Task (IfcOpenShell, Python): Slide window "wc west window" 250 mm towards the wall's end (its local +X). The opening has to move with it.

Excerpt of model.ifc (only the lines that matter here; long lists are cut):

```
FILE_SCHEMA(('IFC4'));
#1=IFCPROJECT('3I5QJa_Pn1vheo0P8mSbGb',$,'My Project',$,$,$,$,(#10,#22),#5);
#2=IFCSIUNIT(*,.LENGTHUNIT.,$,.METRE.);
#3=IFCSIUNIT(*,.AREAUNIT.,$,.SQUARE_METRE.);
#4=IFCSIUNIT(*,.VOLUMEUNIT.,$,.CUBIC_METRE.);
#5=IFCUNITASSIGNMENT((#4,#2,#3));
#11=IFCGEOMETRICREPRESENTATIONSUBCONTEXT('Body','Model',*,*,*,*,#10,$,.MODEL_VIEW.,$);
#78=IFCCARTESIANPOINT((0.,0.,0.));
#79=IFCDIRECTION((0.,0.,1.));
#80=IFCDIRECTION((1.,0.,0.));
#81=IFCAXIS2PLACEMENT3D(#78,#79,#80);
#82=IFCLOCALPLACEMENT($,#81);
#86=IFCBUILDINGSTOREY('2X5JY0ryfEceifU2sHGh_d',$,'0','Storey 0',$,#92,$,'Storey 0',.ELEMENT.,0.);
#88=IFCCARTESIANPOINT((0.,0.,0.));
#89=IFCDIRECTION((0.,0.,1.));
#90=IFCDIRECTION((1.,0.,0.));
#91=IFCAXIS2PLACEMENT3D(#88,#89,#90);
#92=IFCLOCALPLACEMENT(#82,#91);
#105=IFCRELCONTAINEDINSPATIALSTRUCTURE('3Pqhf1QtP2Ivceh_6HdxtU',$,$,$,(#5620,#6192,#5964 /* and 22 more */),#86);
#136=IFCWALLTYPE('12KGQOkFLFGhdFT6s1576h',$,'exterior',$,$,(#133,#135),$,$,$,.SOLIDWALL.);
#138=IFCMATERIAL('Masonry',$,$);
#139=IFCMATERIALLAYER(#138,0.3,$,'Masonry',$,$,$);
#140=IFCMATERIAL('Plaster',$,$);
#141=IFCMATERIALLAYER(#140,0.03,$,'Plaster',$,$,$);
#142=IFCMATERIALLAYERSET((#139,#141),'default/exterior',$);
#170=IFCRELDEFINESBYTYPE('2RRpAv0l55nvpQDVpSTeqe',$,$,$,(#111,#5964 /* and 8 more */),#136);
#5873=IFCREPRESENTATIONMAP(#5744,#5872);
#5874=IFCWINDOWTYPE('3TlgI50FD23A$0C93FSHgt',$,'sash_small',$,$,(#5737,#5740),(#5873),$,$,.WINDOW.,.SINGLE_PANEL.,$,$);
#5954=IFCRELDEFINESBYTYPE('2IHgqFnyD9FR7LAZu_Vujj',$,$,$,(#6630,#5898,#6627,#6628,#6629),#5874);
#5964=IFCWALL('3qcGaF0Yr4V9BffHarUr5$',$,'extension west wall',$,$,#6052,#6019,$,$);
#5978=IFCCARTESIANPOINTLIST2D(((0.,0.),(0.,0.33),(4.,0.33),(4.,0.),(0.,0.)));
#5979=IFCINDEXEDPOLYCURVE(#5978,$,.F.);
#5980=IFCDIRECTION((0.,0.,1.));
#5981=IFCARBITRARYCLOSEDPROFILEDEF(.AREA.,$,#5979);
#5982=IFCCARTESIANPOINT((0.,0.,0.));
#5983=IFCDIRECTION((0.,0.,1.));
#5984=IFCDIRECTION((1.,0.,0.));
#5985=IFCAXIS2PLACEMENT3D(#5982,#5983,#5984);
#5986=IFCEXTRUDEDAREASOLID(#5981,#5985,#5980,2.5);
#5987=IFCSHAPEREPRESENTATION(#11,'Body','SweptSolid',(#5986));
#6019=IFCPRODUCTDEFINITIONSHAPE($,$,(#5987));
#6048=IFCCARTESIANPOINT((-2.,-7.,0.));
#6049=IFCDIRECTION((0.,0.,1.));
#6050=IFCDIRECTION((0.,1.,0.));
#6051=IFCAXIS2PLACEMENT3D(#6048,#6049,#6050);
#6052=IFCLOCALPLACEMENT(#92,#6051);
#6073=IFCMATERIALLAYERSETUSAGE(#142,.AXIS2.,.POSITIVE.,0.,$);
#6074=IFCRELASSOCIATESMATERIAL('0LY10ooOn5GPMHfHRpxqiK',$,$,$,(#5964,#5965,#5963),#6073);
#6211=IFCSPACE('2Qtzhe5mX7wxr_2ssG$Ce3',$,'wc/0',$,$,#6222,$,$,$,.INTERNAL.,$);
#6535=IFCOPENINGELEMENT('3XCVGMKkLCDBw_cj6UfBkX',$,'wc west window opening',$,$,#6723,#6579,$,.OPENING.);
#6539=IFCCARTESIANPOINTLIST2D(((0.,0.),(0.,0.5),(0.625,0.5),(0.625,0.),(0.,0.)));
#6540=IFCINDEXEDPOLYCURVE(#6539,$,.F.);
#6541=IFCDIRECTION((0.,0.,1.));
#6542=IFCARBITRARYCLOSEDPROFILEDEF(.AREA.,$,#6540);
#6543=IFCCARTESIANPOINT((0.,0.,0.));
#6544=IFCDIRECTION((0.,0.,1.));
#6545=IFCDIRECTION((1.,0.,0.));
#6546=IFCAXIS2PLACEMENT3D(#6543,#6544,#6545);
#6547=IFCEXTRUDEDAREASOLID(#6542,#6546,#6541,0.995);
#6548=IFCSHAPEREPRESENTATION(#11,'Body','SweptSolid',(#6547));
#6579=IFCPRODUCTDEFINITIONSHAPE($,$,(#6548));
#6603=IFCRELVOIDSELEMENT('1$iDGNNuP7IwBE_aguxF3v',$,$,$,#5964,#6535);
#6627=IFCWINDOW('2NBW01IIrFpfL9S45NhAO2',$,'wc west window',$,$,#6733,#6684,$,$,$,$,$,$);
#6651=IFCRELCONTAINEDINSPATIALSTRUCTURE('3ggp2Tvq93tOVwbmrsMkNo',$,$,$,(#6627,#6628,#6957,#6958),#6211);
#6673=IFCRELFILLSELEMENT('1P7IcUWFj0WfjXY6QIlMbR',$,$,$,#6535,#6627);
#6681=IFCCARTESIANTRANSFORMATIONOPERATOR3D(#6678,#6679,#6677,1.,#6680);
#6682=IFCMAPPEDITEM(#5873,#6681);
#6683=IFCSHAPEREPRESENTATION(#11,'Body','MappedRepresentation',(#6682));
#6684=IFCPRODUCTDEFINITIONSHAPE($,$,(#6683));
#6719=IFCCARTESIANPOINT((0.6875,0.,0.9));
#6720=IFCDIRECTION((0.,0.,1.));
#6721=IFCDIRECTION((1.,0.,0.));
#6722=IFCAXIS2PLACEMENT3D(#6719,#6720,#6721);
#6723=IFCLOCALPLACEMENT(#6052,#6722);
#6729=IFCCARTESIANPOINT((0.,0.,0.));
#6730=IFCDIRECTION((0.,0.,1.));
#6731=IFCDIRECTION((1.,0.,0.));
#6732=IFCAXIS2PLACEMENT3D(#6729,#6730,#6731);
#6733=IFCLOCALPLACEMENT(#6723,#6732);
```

```python
import ifcopenshell
import ifcopenshell.api.geometry
import ifcopenshell.util.placement

model = ifcopenshell.open("model.ifc")

window = model.by_guid("2NBW01IIrFpfL9S45NhAO2")
opening = window.FillsVoids[0].RelatingOpeningElement
wall = opening.VoidsElements[0].RelatingBuildingElement

wall_matrix = ifcopenshell.util.placement.get_local_placement(wall.ObjectPlacement)
shift = wall_matrix[:3, 0] * 0.25
before = ifcopenshell.util.placement.get_local_placement(window.ObjectPlacement)[:3, 3].copy()

# The window is placed relative to its opening, so it follows when the opening moves.
matrix = ifcopenshell.util.placement.get_local_placement(opening.ObjectPlacement)
matrix[:3, 3] += shift
ifcopenshell.api.geometry.edit_object_placement(
    model, product=opening, matrix=matrix, is_si=False, should_transform_children=True
)

after = ifcopenshell.util.placement.get_local_placement(window.ObjectPlacement)[:3, 3]
print("window moved by", (after - before).round(3) + 0.0)

model.write("model_v2.ifc")
```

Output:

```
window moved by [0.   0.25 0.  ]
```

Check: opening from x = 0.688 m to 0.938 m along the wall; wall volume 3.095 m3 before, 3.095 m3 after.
